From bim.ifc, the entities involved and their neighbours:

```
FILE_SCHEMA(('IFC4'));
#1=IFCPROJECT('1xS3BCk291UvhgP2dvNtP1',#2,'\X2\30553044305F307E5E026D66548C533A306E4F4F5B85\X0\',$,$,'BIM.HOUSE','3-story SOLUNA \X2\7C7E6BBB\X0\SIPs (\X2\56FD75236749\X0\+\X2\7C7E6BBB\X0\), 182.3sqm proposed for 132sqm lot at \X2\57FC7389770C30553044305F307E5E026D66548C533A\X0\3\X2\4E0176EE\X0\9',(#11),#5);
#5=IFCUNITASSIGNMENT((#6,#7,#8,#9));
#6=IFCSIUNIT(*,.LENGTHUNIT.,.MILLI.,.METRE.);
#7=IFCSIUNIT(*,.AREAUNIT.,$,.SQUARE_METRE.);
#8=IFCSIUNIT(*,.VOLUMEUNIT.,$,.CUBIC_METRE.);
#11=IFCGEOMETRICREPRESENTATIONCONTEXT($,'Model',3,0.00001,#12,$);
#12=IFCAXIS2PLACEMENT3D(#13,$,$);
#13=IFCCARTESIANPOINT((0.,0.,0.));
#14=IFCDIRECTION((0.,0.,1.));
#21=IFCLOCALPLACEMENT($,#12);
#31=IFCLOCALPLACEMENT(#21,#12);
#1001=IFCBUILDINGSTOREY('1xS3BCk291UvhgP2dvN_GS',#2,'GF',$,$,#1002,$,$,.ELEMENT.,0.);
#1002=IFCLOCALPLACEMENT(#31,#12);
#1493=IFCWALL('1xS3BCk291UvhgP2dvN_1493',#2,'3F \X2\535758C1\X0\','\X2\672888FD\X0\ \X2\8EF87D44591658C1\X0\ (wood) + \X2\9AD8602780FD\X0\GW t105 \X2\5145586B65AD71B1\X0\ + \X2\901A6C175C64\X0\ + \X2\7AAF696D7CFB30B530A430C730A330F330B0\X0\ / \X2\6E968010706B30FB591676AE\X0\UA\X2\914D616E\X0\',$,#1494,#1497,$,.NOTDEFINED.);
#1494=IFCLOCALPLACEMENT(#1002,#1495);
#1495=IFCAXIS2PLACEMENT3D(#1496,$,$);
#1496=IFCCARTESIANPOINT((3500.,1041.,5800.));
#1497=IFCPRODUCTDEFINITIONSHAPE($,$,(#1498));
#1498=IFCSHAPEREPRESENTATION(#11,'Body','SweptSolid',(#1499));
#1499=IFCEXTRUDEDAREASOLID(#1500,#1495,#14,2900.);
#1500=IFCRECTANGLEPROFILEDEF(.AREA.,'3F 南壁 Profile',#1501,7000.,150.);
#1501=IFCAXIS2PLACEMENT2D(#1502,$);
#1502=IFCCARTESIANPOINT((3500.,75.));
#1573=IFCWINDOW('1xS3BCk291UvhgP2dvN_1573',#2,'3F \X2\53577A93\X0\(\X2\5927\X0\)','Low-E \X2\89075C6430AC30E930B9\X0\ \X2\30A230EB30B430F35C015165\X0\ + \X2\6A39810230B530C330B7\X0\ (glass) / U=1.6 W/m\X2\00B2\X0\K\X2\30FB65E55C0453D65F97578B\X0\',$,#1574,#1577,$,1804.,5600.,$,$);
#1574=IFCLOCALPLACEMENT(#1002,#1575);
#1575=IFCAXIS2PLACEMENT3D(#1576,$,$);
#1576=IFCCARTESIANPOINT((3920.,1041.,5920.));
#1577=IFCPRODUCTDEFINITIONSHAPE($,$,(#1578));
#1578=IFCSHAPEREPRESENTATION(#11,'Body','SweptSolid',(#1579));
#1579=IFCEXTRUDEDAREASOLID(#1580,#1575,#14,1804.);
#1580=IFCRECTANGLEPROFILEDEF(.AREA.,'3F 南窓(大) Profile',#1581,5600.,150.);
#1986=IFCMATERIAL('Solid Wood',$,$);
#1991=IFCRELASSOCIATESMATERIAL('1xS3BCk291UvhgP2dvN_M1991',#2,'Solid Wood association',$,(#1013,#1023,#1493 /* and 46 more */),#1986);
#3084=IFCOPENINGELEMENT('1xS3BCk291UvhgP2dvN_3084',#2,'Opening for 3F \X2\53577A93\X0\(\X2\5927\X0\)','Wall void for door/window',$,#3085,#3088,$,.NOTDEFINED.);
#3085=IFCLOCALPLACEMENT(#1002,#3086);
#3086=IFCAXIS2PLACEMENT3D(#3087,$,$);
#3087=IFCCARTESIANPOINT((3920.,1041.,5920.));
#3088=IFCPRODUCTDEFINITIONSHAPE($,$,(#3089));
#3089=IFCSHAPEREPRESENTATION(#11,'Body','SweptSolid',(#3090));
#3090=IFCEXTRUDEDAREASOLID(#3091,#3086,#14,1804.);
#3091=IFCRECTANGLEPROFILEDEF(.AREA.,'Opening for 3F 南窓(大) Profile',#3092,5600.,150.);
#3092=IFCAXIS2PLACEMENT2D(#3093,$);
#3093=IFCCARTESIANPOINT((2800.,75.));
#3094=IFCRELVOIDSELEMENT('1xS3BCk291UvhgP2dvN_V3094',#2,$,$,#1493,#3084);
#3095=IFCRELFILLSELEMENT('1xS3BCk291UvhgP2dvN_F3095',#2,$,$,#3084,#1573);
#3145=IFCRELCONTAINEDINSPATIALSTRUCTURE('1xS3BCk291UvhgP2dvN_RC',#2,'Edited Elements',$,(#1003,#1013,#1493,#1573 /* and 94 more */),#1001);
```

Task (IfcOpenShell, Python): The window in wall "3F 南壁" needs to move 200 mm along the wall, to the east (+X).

```python
import ifcopenshell
import ifcopenshell.api.geometry
import ifcopenshell.util.placement

model = ifcopenshell.open("bim.ifc")

window = model.by_id(1573)
opening = window.FillsVoids[0].RelatingOpeningElement
wall = opening.VoidsElements[0].RelatingBuildingElement

wall_matrix = ifcopenshell.util.placement.get_local_placement(wall.ObjectPlacement)
shift = wall_matrix[:3, 0] * 200.0
before = ifcopenshell.util.placement.get_local_placement(window.ObjectPlacement)[:3, 3].copy()

# The window is not placed relative to its opening, so move both.
for product in (opening, window):
    matrix = ifcopenshell.util.placement.get_local_placement(product.ObjectPlacement)
    matrix[:3, 3] += shift
    ifcopenshell.api.geometry.edit_object_placement(model, product=product, matrix=matrix, is_si=False)

after = ifcopenshell.util.placement.get_local_placement(window.ObjectPlacement)[:3, 3]
print("window moved by", (after - before).round(3) + 0.0)

model.write("bim_updated.ifc")
```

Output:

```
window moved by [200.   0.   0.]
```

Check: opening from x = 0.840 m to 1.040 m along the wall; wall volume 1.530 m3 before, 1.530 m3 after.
